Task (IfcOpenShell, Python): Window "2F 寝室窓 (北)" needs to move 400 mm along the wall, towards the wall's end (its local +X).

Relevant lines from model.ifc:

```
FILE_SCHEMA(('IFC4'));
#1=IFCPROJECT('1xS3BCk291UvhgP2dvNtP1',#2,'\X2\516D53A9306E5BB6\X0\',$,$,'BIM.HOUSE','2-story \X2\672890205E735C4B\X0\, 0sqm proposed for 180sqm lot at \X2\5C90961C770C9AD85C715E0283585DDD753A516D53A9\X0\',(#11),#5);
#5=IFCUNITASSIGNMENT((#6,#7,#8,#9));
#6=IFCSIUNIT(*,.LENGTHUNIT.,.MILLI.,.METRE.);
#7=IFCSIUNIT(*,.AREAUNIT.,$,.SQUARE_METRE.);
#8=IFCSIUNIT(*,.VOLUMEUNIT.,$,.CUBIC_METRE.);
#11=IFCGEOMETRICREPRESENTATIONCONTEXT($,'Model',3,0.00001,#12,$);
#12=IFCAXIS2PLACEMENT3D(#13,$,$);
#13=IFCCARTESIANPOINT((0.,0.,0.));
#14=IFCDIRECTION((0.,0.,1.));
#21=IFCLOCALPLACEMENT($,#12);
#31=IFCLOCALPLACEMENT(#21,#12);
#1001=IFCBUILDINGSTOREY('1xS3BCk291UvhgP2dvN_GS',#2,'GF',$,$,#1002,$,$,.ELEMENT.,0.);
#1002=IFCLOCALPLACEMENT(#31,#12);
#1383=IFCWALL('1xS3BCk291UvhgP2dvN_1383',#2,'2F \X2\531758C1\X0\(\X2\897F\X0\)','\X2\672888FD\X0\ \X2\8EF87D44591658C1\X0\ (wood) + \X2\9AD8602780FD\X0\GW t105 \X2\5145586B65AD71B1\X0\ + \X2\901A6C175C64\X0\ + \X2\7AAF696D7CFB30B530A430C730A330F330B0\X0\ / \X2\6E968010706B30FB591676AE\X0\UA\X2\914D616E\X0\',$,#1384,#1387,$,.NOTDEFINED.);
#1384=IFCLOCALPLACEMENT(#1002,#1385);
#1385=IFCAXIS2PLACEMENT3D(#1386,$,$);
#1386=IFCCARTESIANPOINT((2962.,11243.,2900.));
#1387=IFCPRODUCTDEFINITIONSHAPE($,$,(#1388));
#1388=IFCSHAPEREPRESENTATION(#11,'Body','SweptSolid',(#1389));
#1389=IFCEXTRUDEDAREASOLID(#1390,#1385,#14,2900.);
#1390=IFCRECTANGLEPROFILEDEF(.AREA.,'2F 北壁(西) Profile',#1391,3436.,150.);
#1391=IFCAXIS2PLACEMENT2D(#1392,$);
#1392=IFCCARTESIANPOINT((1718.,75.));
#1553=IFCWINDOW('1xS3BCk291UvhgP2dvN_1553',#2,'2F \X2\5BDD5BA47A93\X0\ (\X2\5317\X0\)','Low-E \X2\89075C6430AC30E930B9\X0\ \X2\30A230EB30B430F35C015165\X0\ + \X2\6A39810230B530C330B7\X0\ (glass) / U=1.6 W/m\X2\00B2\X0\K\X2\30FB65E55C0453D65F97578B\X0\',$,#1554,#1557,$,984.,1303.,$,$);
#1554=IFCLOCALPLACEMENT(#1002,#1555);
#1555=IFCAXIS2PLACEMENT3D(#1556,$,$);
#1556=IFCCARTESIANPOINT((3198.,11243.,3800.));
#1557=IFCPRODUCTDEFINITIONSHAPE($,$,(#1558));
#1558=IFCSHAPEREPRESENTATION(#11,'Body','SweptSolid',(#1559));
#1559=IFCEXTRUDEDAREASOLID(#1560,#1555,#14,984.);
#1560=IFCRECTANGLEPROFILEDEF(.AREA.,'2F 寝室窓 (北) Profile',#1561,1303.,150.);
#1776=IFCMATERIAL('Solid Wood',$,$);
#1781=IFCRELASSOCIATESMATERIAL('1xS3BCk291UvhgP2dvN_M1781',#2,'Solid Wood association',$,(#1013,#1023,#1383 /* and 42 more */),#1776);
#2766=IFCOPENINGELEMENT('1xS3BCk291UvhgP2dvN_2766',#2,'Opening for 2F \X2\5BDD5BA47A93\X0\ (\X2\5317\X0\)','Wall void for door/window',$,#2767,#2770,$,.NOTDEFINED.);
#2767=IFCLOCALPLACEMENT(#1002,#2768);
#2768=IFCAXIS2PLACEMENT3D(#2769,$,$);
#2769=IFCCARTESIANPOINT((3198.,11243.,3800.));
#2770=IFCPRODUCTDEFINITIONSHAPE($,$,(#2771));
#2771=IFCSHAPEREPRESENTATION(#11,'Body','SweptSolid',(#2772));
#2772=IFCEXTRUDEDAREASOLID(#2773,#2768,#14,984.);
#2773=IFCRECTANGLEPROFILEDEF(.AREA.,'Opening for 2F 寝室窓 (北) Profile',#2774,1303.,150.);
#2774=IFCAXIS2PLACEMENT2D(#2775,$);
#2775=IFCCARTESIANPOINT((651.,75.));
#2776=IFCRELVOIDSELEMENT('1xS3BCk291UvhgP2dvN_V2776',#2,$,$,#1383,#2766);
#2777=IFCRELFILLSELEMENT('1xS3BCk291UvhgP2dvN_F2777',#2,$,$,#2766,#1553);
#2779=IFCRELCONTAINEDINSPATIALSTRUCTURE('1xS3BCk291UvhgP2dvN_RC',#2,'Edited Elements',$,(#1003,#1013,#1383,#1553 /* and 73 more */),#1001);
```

```python
import ifcopenshell
import ifcopenshell.api.geometry
import ifcopenshell.util.placement
import ifcopenshell.util.unit

model = ifcopenshell.open("model.ifc")
unit_scale = ifcopenshell.util.unit.calculate_unit_scale(model)

window = model.by_id(1553)
opening = window.FillsVoids[0].RelatingOpeningElement
wall = opening.VoidsElements[0].RelatingBuildingElement

wall_matrix = ifcopenshell.util.placement.get_local_placement(wall.ObjectPlacement)
shift = wall_matrix[:3, 0] * 0.4 / unit_scale
before = ifcopenshell.util.placement.get_local_placement(window.ObjectPlacement)[:3, 3].copy()

# The window is not placed relative to its opening, so move both.
for product in (opening, window):
    matrix = ifcopenshell.util.placement.get_local_placement(product.ObjectPlacement)
    matrix[:3, 3] += shift
    ifcopenshell.api.geometry.edit_object_placement(model, product=product, matrix=matrix, is_si=False)

after = ifcopenshell.util.placement.get_local_placement(window.ObjectPlacement)[:3, 3]
print("window moved by", (after - before).round(3) + 0.0)

model.write("model_updated.ifc")
```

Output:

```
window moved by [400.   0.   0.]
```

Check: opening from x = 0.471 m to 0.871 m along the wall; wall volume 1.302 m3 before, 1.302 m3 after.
